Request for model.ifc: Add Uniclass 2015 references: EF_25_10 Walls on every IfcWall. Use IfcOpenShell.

First a look at what the model holds.

```python
import ifcopenshell

model = ifcopenshell.open("model.ifc")
print(model.schema)
print("classifications:", [c.Name for c in model.by_type("IfcClassification")])
for ifc_class in ("IfcDoor", "IfcRoof", "IfcStair", "IfcWall", "IfcWindow"):
    print(ifc_class, len(model.by_type(ifc_class)))
```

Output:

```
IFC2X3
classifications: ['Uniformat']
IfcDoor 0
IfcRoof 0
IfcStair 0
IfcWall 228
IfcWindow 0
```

```python
import ifcopenshell
import ifcopenshell.api.classification

model = ifcopenshell.open("model.ifc")

# IFC2X3 requires Source and Edition and has no link from the project to the system.
system = model.create_entity("IfcClassification", Source="NBS", Edition="2015", Name="Uniclass 2015")

codes = {
    "IfcWall": ("EF_25_10", "Walls"),
}
for ifc_class, (code, name) in codes.items():
    products = model.by_type(ifc_class)
    ifcopenshell.api.classification.add_reference(
        model, products=products, classification=system, identification=code, name=name
    )
    print(code, len(products))

model.write("model_edited.ifc")
```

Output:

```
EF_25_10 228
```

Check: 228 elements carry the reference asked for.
